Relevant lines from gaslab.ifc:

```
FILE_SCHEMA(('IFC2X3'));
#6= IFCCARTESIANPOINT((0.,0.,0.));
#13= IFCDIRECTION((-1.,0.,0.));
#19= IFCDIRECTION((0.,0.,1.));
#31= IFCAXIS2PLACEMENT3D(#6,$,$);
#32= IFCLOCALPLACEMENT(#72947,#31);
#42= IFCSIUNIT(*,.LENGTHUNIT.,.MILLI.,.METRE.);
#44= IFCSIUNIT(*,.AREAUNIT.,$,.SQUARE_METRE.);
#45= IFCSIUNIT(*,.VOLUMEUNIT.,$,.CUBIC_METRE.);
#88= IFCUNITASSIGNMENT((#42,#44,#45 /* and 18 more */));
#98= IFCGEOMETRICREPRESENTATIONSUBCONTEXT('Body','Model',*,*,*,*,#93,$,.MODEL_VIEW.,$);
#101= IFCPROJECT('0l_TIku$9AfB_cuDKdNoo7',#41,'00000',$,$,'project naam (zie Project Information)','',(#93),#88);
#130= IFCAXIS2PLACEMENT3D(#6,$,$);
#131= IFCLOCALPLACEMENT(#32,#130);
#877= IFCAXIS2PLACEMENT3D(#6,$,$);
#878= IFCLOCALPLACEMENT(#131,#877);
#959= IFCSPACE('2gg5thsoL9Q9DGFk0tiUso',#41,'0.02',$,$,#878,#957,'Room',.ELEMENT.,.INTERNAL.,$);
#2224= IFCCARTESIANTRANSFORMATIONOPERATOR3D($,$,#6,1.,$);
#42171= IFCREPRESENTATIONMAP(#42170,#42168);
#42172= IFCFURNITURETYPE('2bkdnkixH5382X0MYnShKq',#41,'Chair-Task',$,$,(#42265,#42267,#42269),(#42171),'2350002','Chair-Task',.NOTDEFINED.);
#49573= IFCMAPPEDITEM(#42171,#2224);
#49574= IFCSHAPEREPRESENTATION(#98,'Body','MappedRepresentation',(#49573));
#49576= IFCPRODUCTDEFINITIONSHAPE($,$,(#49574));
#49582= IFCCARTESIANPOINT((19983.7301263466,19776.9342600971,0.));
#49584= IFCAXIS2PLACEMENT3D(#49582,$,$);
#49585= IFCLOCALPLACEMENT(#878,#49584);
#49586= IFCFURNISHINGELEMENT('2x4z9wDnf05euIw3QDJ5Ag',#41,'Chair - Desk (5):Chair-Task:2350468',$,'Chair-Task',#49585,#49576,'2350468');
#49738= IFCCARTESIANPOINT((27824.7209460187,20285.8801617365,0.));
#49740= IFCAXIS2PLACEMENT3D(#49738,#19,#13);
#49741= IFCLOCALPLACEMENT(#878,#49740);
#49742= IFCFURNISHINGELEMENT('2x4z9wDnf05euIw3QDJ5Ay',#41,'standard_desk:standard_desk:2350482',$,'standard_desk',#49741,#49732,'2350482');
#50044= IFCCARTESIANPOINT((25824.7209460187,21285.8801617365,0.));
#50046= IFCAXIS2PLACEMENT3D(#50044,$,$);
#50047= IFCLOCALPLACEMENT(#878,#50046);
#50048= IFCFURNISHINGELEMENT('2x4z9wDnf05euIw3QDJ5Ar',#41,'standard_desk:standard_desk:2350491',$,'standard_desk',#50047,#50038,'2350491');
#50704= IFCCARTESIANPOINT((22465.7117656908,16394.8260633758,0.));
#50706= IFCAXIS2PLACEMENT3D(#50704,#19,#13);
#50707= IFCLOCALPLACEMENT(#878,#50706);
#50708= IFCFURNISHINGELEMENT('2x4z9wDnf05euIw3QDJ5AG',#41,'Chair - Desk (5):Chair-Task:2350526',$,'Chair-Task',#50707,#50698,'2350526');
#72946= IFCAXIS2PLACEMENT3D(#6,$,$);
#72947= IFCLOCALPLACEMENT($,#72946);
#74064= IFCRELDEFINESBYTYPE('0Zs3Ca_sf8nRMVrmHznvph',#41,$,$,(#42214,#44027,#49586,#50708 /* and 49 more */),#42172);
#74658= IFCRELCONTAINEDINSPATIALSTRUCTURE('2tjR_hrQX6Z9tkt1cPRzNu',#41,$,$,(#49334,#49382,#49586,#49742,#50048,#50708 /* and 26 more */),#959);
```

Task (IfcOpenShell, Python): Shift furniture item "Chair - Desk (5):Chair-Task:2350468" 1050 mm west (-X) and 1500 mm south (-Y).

```python
import ifcopenshell
import ifcopenshell.api.geometry
import ifcopenshell.util.placement
import ifcopenshell.util.unit

model = ifcopenshell.open("gaslab.ifc")
unit_scale = ifcopenshell.util.unit.calculate_unit_scale(model)

item = model.by_id(49586)
matrix = ifcopenshell.util.placement.get_local_placement(item.ObjectPlacement)
matrix[0, 3] -= 1.05 / unit_scale
matrix[1, 3] -= 1.5 / unit_scale
ifcopenshell.api.geometry.edit_object_placement(model, product=item, matrix=matrix, is_si=False)

print(ifcopenshell.util.placement.get_local_placement(item.ObjectPlacement).round(3) + 0.0)

model.write("gaslab_edited.ifc")
```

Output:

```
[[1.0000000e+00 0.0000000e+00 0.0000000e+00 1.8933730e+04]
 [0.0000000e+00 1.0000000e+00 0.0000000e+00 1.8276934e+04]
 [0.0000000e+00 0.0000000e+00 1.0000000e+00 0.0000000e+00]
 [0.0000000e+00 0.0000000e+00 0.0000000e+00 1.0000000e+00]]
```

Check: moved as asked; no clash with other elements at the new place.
